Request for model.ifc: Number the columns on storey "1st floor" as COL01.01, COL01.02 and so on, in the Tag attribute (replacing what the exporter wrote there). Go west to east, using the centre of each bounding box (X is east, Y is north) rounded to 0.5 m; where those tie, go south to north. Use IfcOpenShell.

First a look at what the model holds.

```python
import ifcopenshell
import ifcopenshell.util.element
import ifcopenshell.util.placement

model = ifcopenshell.open("model.ifc")
print(model.schema)
storey = next(s for s in model.by_type("IfcBuildingStorey") if s.Name == "1st floor")
columns = [e for e in ifcopenshell.util.element.get_decomposition(storey) if e.is_a("IfcColumn")]
for e in sorted(columns, key=lambda e: e.id()):
    origin = ifcopenshell.util.placement.get_local_placement(e.ObjectPlacement)[:3, 3]
    print(e.id(), e.Tag, e.Name, origin.round(2) + 0.0, sep=" | ")
```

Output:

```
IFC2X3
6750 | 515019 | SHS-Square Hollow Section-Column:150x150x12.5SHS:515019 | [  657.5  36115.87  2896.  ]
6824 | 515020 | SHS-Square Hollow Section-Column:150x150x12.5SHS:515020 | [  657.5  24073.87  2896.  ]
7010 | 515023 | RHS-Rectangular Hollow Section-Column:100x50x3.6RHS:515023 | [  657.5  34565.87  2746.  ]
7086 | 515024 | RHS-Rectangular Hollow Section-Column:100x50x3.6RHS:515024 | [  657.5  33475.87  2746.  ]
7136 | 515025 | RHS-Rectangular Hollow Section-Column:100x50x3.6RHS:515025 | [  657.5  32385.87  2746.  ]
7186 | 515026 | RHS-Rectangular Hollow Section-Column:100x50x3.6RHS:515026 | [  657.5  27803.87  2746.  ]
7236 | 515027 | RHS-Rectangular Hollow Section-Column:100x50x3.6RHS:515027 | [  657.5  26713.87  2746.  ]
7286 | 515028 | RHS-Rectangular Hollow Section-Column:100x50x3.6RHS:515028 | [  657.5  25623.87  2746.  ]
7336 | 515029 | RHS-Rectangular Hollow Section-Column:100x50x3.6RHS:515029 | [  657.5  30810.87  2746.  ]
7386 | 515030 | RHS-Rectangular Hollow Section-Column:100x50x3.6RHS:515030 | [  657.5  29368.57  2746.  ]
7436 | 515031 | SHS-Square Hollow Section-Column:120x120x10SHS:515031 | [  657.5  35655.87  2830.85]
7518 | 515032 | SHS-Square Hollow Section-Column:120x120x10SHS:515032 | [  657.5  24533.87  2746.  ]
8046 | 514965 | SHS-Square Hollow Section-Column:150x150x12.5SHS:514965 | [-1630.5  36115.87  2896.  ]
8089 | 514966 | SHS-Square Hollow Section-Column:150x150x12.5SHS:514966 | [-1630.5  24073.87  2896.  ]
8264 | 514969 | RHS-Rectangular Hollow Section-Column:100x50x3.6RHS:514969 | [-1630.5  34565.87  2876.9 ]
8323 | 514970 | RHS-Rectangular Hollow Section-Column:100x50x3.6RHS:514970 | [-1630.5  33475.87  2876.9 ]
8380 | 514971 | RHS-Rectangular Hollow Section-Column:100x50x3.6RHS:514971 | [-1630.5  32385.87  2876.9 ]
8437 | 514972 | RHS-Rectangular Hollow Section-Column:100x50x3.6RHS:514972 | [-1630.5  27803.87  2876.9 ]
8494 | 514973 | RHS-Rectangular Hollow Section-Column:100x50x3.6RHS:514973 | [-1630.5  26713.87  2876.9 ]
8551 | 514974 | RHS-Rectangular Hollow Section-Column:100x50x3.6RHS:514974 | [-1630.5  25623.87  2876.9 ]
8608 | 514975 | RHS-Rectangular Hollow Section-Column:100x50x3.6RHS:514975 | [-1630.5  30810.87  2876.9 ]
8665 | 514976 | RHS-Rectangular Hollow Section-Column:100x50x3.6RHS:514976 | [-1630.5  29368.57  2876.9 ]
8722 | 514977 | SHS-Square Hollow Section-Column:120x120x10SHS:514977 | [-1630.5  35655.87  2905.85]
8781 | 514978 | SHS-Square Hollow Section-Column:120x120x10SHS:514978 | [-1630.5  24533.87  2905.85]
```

```python
import ifcopenshell
import ifcopenshell.geom
import ifcopenshell.util.element
import ifcopenshell.util.shape

model = ifcopenshell.open("model.ifc")
settings = ifcopenshell.geom.settings()
settings.set("use-world-coords", True)


def centre(element):
    shape = ifcopenshell.geom.create_shape(settings, element)
    return ifcopenshell.util.shape.get_bbox_centroid(shape.geometry)


storey = next(s for s in model.by_type("IfcBuildingStorey") if s.Name == "1st floor")
columns = [e for e in ifcopenshell.util.element.get_decomposition(storey) if e.is_a("IfcColumn")]

# Insertion points can sit at a corner or the storey origin, so sort by the geometry (in metres).
centres = {e: centre(e) for e in columns}
columns.sort(key=lambda e: (round(centres[e][0] / 0.5), centres[e][1]))

for i, e in enumerate(columns, start=1):
    number = f"COL01.{i:02d}"
    e.Tag = number
    print(e.id(), number)

model.write("model-out.ifc")
```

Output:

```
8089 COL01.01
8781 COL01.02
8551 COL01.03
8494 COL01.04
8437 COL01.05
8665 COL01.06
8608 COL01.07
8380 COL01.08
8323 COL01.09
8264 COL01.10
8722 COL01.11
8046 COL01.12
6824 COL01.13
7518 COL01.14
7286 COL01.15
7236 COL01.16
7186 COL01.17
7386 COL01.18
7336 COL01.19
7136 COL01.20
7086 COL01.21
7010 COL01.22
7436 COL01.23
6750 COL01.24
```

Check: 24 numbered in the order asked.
